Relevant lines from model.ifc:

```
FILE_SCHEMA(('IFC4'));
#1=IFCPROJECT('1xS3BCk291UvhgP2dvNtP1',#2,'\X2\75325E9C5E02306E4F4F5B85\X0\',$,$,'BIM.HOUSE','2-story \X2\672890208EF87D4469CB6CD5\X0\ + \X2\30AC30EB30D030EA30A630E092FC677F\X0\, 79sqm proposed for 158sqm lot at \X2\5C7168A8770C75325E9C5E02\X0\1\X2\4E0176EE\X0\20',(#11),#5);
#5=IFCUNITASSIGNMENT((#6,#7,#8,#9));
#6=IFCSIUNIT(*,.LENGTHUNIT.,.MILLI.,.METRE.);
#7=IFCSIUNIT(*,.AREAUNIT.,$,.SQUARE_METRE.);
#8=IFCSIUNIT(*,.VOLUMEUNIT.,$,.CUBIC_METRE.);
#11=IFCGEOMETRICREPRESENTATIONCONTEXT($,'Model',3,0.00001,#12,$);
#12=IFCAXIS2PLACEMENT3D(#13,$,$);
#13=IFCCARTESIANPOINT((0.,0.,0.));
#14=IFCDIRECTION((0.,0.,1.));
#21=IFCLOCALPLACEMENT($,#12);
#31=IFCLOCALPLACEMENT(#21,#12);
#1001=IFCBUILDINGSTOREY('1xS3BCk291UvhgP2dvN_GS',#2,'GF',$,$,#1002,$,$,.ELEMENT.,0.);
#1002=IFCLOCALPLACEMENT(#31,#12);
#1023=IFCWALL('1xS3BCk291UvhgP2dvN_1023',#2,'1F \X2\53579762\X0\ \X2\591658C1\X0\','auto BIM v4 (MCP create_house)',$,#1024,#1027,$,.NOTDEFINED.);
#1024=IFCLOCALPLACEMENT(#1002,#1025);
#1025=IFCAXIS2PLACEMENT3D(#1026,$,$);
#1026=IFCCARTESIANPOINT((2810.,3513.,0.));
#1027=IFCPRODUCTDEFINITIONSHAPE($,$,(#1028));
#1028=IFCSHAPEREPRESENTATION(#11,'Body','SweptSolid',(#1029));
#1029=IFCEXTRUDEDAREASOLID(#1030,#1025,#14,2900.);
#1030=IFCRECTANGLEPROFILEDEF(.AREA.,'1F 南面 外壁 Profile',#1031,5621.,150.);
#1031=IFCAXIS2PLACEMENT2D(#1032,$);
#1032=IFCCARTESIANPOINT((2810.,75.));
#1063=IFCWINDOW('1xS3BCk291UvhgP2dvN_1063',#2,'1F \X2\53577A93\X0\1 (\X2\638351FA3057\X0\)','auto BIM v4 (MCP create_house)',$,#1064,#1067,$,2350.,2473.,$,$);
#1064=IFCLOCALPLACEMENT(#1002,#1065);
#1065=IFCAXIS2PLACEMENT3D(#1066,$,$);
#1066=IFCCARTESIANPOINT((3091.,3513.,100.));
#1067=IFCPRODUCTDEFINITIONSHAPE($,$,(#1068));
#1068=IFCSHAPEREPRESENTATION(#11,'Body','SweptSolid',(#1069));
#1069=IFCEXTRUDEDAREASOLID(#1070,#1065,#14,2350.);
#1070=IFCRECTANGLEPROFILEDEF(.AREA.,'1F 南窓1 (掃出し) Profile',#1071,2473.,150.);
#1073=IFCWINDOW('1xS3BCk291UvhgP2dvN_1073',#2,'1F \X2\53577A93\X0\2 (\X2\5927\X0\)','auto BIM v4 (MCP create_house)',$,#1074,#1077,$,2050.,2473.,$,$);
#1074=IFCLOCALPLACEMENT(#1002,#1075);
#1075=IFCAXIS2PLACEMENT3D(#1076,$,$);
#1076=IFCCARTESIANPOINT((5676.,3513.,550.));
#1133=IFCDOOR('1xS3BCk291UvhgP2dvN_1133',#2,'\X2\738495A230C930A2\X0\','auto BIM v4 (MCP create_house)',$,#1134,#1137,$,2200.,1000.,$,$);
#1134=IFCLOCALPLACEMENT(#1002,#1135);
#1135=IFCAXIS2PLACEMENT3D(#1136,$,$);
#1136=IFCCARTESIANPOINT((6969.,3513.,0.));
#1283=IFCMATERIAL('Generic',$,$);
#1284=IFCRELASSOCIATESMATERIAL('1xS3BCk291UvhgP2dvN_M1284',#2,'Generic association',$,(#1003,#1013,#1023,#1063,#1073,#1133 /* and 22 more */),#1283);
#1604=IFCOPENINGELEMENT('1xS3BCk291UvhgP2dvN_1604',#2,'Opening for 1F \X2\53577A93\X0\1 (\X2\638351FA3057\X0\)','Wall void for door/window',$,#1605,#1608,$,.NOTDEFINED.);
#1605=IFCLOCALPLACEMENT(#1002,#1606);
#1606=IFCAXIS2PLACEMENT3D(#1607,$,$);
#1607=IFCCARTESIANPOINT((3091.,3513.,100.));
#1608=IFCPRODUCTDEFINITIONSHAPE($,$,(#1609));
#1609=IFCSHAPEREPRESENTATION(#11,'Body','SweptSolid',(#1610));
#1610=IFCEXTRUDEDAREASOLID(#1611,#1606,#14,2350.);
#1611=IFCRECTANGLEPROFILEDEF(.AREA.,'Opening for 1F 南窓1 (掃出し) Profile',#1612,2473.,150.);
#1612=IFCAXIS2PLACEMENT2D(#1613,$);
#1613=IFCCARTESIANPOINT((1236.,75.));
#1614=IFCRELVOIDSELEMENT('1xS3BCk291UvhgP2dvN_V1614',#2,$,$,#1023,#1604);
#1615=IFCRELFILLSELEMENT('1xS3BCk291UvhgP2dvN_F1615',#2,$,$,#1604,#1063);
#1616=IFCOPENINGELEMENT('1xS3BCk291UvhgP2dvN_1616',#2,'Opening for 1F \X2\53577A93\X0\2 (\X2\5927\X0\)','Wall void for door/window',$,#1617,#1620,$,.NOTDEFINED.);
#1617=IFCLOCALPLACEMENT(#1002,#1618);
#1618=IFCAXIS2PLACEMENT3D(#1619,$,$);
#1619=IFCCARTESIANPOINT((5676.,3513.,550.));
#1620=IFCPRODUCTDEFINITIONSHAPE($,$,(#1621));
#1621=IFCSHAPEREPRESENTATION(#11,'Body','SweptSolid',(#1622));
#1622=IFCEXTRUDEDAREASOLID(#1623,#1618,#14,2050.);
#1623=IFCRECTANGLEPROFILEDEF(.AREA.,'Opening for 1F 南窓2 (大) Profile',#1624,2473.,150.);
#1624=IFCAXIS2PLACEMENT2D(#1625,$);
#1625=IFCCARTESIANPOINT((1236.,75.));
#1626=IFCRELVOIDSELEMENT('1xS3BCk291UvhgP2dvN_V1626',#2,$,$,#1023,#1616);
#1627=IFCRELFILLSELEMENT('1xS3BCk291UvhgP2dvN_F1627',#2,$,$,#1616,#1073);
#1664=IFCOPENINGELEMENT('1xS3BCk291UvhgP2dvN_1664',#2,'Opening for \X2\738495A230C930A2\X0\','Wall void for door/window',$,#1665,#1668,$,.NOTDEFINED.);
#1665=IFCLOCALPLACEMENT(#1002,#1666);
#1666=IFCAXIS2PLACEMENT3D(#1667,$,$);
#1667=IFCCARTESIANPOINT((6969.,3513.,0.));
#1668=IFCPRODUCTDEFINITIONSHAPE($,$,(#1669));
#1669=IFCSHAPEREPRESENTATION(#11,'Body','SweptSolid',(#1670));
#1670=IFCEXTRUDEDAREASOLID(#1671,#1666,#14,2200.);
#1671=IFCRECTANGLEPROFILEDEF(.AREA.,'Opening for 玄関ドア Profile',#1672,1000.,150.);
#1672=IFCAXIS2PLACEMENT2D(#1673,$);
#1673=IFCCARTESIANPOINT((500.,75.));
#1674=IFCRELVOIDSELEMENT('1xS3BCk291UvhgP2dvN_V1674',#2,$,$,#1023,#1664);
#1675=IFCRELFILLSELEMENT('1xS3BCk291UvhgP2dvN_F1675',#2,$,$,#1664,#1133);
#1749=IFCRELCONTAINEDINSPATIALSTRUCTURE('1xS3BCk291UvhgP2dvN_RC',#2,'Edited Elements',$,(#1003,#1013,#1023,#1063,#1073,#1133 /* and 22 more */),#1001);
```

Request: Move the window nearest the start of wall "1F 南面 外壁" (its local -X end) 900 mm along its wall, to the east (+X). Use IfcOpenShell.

```python
import ifcopenshell
import ifcopenshell.api.geometry
import ifcopenshell.util.placement
import ifcopenshell.util.unit

model = ifcopenshell.open("model.ifc")
unit_scale = ifcopenshell.util.unit.calculate_unit_scale(model)

window = model.by_guid("1xS3BCk291UvhgP2dvN_1063")
opening = window.FillsVoids[0].RelatingOpeningElement
wall = opening.VoidsElements[0].RelatingBuildingElement

wall_matrix = ifcopenshell.util.placement.get_local_placement(wall.ObjectPlacement)
shift = wall_matrix[:3, 0] * 0.9 / unit_scale
before = ifcopenshell.util.placement.get_local_placement(window.ObjectPlacement)[:3, 3].copy()

# The window is not placed relative to its opening, so move both.
for product in (opening, window):
    matrix = ifcopenshell.util.placement.get_local_placement(product.ObjectPlacement)
    matrix[:3, 3] += shift
    ifcopenshell.api.geometry.edit_object_placement(model, product=product, matrix=matrix, is_si=False)

after = ifcopenshell.util.placement.get_local_placement(window.ObjectPlacement)[:3, 3]
print("window moved by", (after - before).round(3) + 0.0)

model.write("model_v2.ifc")
```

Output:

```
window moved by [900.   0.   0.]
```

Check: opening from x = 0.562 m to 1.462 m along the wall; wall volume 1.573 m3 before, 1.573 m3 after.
